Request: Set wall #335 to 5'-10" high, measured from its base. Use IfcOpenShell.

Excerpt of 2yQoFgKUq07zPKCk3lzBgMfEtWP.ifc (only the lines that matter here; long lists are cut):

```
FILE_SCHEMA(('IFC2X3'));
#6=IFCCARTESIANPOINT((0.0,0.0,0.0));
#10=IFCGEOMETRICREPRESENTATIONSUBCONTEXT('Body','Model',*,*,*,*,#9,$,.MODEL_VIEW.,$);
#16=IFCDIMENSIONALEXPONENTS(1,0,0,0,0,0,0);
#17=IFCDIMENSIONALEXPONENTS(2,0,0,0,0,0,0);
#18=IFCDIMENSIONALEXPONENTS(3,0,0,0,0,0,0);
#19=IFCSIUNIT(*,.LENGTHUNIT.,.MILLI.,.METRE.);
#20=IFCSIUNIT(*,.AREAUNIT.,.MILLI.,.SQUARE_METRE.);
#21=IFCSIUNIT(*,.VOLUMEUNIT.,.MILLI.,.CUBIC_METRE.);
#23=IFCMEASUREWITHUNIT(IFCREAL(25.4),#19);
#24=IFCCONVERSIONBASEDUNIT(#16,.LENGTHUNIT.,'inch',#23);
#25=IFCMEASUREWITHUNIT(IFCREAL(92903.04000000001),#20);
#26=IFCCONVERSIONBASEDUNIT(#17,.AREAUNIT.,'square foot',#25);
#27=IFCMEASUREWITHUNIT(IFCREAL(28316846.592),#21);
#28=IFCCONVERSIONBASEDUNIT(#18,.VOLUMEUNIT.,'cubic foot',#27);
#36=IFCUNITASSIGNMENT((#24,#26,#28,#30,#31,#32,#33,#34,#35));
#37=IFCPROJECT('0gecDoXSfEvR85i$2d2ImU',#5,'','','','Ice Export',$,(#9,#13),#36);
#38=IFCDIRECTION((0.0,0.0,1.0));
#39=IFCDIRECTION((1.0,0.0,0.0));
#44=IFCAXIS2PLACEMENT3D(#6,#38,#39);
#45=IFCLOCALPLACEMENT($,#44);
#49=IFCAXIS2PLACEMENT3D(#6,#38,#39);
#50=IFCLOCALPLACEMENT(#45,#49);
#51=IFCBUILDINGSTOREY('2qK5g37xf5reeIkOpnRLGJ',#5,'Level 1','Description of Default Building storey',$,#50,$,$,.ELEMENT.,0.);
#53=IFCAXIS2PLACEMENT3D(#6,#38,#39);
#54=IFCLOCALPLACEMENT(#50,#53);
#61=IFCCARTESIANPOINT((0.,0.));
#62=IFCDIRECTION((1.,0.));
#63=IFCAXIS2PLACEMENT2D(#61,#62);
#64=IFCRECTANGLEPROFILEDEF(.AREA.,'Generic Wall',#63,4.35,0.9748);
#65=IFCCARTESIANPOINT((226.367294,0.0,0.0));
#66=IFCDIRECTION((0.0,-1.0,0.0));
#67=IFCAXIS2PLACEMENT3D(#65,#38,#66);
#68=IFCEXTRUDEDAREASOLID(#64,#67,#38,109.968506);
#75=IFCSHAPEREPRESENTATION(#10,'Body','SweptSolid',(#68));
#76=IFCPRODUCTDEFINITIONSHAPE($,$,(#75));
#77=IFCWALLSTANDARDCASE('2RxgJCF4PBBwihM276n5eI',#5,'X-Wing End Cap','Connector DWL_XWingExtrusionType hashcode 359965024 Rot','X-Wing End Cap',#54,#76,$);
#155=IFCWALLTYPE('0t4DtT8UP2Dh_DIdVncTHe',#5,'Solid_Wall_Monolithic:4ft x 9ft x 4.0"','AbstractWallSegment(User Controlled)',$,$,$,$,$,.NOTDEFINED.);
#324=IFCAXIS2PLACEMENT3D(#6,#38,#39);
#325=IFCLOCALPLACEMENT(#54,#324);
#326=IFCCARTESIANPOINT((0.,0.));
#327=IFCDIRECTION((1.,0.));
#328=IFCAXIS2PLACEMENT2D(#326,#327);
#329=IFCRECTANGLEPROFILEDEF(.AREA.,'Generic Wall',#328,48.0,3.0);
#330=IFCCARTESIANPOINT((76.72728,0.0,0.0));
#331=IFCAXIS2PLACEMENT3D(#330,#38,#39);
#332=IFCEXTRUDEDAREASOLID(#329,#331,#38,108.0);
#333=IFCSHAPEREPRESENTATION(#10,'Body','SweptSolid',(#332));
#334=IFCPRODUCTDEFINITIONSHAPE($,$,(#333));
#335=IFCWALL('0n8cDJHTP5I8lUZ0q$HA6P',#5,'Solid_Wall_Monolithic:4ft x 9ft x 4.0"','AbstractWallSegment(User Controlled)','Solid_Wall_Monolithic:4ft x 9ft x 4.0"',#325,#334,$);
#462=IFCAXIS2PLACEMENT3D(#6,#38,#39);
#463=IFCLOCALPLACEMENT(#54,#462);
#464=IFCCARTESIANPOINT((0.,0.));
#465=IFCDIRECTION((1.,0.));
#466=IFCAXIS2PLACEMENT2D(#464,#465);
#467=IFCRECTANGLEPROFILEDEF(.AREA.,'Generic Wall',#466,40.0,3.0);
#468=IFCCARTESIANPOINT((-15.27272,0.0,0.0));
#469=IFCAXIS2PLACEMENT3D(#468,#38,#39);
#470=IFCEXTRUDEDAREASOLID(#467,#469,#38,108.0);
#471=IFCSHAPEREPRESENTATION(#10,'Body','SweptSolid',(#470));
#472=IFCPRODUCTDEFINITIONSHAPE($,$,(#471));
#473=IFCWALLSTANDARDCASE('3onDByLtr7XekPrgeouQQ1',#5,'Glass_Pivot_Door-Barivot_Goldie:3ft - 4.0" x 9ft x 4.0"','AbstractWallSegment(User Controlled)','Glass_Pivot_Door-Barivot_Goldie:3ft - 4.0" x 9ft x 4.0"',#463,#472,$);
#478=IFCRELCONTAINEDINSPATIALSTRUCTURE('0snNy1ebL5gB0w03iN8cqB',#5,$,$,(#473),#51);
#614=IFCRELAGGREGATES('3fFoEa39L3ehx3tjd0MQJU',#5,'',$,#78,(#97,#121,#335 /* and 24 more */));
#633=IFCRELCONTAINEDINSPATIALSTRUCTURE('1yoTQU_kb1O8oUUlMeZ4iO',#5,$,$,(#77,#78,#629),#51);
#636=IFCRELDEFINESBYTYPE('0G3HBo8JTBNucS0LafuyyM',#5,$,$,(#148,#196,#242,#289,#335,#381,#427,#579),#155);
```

```python
import ifcopenshell
import ifcopenshell.geom
import ifcopenshell.util.representation
import ifcopenshell.util.shape
import ifcopenshell.util.unit

model = ifcopenshell.open("2yQoFgKUq07zPKCk3lzBgMfEtWP.ifc")
unit_scale = ifcopenshell.util.unit.calculate_unit_scale(model)
settings = ifcopenshell.geom.settings()


def volume(element):
    """Net volume in cubic metres, openings subtracted."""
    shape = ifcopenshell.geom.create_shape(settings, element)
    return ifcopenshell.util.shape.get_volume(shape.geometry)


wall = model.by_id(335)
before = volume(wall)

body = ifcopenshell.util.representation.get_representation(wall, "Model", "Body")
solid = body.Items[0]
old_height = solid.Depth
solid.Depth = 70 * 0.0254 / unit_scale
after = volume(wall)

print(f"height {old_height:g} -> {solid.Depth:g}, volume {before:.3f} -> {after:.3f} m3")

model.write("2yQoFgKUq07zPKCk3lzBgMfEtWP_updated.ifc")
```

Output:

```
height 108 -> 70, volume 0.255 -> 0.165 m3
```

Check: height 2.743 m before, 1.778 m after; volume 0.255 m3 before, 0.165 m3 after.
